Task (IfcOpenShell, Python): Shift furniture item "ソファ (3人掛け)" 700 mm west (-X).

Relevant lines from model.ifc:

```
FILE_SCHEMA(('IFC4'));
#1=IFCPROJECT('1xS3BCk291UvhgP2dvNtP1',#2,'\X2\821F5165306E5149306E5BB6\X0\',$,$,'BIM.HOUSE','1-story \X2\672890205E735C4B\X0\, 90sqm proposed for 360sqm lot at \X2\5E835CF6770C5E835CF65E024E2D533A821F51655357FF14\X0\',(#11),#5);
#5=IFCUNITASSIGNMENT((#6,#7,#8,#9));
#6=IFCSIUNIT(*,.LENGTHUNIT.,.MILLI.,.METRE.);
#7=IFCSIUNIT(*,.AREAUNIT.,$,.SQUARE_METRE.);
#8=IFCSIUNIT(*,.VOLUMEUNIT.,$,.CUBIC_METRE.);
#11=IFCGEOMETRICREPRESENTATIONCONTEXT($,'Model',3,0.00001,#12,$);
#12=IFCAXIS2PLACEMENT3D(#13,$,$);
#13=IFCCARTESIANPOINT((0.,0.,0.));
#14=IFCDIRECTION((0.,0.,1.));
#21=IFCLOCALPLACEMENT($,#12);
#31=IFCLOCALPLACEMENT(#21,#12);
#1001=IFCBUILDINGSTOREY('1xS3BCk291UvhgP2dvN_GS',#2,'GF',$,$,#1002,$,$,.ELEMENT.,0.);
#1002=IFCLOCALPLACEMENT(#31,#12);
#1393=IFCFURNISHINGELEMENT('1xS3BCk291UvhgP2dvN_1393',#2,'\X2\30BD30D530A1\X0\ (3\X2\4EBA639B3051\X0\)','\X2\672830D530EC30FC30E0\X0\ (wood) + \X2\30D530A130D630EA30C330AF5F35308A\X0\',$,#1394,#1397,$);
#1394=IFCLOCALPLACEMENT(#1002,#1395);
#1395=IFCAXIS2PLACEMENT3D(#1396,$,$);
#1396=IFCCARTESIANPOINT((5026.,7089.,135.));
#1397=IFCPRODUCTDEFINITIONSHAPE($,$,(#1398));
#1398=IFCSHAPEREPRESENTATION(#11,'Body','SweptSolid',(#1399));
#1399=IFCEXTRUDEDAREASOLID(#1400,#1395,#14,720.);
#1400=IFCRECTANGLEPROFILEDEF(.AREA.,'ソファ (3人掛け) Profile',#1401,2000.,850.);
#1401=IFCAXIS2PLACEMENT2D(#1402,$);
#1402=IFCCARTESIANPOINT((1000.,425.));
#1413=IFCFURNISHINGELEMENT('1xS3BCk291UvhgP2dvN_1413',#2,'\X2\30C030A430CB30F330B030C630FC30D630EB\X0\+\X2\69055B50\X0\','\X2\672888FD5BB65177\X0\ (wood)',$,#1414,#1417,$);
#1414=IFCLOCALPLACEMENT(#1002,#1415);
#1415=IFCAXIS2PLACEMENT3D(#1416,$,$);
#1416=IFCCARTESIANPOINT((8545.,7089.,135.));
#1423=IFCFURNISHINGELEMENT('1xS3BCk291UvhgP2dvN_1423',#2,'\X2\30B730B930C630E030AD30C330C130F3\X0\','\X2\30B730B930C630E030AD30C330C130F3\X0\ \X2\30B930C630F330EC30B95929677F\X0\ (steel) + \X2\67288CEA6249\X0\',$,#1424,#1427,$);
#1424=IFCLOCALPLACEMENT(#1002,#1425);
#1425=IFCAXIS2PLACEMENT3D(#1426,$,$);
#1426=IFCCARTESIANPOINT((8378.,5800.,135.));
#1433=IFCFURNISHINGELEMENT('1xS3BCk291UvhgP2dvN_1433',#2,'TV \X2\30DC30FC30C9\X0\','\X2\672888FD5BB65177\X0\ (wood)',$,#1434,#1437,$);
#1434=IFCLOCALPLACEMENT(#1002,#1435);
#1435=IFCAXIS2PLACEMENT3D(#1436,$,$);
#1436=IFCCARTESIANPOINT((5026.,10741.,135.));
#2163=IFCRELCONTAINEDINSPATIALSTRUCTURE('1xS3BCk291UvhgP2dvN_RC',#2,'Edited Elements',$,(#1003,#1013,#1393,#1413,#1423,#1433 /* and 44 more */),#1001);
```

```python
import ifcopenshell
import ifcopenshell.api.geometry
import ifcopenshell.util.placement
import ifcopenshell.util.unit

model = ifcopenshell.open("model.ifc")
unit_scale = ifcopenshell.util.unit.calculate_unit_scale(model)

item = model.by_guid("1xS3BCk291UvhgP2dvN_1393")
matrix = ifcopenshell.util.placement.get_local_placement(item.ObjectPlacement)
matrix[0, 3] -= 0.7 / unit_scale
ifcopenshell.api.geometry.edit_object_placement(model, product=item, matrix=matrix, is_si=False)

print(ifcopenshell.util.placement.get_local_placement(item.ObjectPlacement).round(3) + 0.0)

model.write("model_edited.ifc")
```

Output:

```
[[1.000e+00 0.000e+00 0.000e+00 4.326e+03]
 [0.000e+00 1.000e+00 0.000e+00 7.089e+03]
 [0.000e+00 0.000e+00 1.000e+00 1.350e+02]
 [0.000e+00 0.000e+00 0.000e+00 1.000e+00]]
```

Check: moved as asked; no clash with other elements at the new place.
